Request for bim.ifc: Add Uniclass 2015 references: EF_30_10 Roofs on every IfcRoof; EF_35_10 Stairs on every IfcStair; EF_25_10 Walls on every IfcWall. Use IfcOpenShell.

First a look at what the model holds.

```python
import ifcopenshell

model = ifcopenshell.open("bim.ifc")
print(model.schema)
print("classifications:", [c.Name for c in model.by_type("IfcClassification")])
for ifc_class in ("IfcDoor", "IfcRoof", "IfcStair", "IfcWall", "IfcWindow"):
    print(ifc_class, len(model.by_type(ifc_class)))
```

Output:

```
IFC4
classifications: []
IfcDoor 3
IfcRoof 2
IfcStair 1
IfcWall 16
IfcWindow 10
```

```python
import ifcopenshell
import ifcopenshell.api.classification

model = ifcopenshell.open("bim.ifc")

system = ifcopenshell.api.classification.add_classification(model, classification="Uniclass 2015")

codes = {
    "IfcRoof": ("EF_30_10", "Roofs"),
    "IfcStair": ("EF_35_10", "Stairs"),
    "IfcWall": ("EF_25_10", "Walls"),
}
for ifc_class, (code, name) in codes.items():
    products = model.by_type(ifc_class)
    ifcopenshell.api.classification.add_reference(
        model, products=products, classification=system, identification=code, name=name
    )
    print(code, len(products))

model.write("bim-out.ifc")
```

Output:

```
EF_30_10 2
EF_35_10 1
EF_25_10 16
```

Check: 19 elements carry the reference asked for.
